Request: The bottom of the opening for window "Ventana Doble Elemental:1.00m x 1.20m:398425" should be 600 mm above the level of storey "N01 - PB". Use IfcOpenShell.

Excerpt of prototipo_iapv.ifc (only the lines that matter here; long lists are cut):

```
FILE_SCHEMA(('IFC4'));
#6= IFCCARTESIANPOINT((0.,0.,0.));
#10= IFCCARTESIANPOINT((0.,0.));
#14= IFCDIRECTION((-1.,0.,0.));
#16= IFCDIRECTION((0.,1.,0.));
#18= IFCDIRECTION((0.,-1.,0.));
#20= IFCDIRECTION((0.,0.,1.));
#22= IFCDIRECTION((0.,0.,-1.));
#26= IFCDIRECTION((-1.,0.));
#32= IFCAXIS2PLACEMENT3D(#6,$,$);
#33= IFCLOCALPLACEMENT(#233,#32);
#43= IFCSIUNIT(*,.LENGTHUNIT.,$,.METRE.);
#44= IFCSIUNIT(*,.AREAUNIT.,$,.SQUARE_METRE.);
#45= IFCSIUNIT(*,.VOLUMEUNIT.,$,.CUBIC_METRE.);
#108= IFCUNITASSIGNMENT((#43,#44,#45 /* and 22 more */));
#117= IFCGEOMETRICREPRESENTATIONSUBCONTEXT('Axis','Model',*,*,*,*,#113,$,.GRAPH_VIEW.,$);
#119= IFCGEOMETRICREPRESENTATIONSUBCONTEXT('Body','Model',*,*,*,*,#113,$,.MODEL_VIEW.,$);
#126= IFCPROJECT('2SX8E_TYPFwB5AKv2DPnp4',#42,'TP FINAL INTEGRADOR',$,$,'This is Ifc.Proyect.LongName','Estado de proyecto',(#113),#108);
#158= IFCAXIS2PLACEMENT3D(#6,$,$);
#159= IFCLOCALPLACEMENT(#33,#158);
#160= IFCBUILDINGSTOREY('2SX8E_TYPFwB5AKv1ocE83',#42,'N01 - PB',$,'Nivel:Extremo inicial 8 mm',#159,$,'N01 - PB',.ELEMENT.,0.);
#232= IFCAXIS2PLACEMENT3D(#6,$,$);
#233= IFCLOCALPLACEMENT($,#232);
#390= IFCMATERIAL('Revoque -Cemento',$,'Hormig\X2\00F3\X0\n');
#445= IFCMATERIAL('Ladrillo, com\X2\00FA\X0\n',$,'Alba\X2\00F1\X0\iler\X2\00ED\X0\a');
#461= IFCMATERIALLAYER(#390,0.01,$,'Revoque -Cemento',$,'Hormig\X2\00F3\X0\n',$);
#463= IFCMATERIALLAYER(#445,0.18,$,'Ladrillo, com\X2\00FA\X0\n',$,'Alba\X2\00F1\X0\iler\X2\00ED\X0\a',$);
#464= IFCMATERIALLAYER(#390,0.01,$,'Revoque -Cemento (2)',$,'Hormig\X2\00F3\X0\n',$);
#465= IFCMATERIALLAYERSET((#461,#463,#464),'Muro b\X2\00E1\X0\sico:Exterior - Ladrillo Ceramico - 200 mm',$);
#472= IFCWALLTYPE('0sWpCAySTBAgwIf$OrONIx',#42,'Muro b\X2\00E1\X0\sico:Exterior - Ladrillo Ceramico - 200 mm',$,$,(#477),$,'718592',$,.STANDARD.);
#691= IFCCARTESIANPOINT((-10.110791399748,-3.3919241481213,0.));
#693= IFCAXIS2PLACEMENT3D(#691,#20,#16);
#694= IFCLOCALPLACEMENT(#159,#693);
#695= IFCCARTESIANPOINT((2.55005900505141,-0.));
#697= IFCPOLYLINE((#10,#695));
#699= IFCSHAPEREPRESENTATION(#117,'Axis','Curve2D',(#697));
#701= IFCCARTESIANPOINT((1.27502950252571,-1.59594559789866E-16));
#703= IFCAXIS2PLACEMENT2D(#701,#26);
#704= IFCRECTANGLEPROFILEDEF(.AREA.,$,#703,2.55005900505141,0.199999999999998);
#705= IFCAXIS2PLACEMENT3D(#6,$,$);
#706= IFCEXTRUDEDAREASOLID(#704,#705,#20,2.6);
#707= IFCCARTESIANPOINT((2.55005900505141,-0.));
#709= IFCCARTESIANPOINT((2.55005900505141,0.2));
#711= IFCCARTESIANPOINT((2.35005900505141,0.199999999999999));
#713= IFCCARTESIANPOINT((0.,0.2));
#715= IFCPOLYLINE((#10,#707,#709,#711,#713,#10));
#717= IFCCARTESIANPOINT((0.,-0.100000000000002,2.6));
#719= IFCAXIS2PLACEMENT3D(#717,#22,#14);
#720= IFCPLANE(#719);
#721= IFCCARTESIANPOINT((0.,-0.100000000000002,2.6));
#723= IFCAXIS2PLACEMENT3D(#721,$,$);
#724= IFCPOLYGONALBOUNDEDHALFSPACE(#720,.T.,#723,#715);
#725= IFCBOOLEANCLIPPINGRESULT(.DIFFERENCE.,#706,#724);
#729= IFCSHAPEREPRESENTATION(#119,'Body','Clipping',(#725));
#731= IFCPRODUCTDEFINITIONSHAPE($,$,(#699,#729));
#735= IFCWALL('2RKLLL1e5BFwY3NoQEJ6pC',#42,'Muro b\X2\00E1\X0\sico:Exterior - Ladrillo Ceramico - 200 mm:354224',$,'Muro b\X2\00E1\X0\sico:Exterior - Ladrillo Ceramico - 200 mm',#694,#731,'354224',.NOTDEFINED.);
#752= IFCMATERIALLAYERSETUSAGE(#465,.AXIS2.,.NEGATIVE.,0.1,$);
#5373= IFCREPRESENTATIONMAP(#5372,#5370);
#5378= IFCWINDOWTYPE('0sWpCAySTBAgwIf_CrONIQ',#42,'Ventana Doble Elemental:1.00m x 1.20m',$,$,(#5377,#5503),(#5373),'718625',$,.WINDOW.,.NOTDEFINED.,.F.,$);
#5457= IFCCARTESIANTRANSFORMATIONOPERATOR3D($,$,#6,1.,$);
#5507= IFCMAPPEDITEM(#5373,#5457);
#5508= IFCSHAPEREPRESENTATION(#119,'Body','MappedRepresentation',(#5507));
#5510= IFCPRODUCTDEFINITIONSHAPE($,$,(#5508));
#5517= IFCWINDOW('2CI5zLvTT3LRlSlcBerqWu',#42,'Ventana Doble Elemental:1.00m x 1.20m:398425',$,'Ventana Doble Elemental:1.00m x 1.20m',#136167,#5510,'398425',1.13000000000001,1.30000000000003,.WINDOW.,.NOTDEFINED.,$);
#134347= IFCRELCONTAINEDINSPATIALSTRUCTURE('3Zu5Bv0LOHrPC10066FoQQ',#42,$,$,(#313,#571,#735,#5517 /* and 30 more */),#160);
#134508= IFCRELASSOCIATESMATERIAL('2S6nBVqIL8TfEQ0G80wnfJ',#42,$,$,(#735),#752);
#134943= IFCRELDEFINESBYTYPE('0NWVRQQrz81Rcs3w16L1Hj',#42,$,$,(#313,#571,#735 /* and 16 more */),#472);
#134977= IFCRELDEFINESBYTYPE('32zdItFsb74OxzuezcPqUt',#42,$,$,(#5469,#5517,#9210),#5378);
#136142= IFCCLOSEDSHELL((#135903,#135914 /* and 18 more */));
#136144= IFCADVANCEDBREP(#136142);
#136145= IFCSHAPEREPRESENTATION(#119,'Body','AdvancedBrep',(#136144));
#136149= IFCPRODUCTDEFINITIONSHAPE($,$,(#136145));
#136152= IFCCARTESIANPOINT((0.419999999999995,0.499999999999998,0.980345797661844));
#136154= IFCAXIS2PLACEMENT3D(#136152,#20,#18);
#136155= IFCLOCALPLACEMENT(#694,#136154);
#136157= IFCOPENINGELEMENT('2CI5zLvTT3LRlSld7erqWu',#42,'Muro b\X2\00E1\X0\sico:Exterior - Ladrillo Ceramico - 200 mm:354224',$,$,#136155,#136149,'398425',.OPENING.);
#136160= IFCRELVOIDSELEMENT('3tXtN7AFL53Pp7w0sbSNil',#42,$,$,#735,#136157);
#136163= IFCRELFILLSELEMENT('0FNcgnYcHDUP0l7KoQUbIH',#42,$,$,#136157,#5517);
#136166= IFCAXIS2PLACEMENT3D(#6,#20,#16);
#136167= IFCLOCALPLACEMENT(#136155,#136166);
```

```python
import numpy as np
import ifcopenshell
import ifcopenshell.api.geometry
import ifcopenshell.geom
import ifcopenshell.util.element
import ifcopenshell.util.placement
import ifcopenshell.util.shape
import ifcopenshell.util.unit

model = ifcopenshell.open("prototipo_iapv.ifc")
unit_scale = ifcopenshell.util.unit.calculate_unit_scale(model)

window = model.by_guid("2CI5zLvTT3LRlSlcBerqWu")
opening = window.FillsVoids[0].RelatingOpeningElement
storey = ifcopenshell.util.element.get_container(window, ifc_class="IfcBuildingStorey")
level = ifcopenshell.util.placement.get_local_placement(storey.ObjectPlacement)[2, 3]

# The opening's origin need not be at the sill, so measure its lowest point.
shape = ifcopenshell.geom.create_shape(ifcopenshell.geom.settings(), opening)
bottom = ifcopenshell.util.shape.get_shape_bottom_elevation(shape, shape.geometry) / unit_scale
dz = level + 0.6 / unit_scale - bottom

shift = np.array([0.0, 0.0, dz])
# The window is placed relative to its opening, so it follows when the opening moves.
matrix = ifcopenshell.util.placement.get_local_placement(opening.ObjectPlacement)
matrix[:3, 3] += shift
ifcopenshell.api.geometry.edit_object_placement(
    model, product=opening, matrix=matrix, is_si=False, should_transform_children=True
)

print(f"moved by {dz * unit_scale:+.3f} m")

model.write("prototipo_iapv_v2.ifc")
```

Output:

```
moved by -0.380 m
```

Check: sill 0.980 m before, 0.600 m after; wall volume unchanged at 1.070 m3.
